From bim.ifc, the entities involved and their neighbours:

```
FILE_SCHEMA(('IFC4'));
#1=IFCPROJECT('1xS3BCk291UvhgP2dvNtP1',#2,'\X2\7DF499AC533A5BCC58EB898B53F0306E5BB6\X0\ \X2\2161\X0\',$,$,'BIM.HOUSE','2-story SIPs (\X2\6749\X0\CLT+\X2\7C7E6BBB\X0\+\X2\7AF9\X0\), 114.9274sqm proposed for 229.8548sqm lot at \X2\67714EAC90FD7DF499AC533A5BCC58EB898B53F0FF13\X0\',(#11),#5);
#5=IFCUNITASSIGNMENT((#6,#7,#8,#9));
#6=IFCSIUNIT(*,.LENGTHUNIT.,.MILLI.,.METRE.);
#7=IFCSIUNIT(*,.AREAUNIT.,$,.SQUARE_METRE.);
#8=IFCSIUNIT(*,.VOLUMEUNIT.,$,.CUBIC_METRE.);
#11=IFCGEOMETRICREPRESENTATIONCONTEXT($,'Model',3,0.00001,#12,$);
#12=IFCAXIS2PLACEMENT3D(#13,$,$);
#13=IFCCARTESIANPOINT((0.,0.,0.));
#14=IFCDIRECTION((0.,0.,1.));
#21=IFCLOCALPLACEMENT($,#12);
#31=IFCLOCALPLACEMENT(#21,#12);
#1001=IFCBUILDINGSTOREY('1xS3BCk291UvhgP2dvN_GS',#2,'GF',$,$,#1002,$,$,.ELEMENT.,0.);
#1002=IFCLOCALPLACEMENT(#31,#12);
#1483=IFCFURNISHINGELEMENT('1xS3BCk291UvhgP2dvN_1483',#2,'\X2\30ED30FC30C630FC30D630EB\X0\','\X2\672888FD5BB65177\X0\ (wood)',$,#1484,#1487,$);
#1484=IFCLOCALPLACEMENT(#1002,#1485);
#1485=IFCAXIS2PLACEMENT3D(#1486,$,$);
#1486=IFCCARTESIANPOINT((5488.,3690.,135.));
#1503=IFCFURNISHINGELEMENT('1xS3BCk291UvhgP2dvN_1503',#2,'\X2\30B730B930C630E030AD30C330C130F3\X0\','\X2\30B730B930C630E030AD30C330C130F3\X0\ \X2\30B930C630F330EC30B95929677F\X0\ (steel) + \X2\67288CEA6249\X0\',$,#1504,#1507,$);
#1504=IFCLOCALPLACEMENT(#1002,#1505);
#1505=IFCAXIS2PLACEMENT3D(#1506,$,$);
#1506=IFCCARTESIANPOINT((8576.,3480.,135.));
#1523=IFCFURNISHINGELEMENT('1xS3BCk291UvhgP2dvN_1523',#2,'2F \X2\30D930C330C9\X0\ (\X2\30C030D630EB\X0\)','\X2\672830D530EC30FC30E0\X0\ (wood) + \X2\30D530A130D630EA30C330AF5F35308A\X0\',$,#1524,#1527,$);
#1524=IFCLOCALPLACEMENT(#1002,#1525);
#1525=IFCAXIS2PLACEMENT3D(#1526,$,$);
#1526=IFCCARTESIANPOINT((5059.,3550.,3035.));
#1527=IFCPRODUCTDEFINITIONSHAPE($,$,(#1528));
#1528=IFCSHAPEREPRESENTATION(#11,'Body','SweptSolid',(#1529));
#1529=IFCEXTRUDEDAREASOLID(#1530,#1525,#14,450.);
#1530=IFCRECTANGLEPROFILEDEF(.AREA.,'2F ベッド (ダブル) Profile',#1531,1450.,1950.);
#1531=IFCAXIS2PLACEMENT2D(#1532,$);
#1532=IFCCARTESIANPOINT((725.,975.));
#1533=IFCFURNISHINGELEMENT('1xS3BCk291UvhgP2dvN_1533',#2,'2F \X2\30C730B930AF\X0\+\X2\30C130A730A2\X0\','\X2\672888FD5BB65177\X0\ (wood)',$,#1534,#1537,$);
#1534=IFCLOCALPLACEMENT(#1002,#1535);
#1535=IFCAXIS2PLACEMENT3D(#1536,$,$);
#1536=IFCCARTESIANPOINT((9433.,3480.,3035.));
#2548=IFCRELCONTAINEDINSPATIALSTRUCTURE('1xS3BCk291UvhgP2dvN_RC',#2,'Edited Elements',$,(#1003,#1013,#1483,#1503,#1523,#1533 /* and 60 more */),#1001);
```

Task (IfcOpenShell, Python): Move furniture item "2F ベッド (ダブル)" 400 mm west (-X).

```python
import ifcopenshell
import ifcopenshell.api.geometry
import ifcopenshell.util.placement
import ifcopenshell.util.unit

model = ifcopenshell.open("bim.ifc")
unit_scale = ifcopenshell.util.unit.calculate_unit_scale(model)

item = model.by_id(1523)
matrix = ifcopenshell.util.placement.get_local_placement(item.ObjectPlacement)
matrix[0, 3] -= 0.4 / unit_scale
ifcopenshell.api.geometry.edit_object_placement(model, product=item, matrix=matrix, is_si=False)

print(ifcopenshell.util.placement.get_local_placement(item.ObjectPlacement).round(3) + 0.0)

model.write("bim_rev.ifc")
```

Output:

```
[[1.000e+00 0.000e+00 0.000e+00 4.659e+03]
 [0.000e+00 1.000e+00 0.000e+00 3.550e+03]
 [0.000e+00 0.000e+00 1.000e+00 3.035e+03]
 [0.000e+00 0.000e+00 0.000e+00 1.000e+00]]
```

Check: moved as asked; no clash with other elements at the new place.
